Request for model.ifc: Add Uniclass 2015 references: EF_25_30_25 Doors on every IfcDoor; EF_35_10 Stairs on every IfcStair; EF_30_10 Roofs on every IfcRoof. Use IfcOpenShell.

First a look at what the model holds.

```python
import ifcopenshell

model = ifcopenshell.open("model.ifc")
print(model.schema)
print("classifications:", [c.Name for c in model.by_type("IfcClassification")])
for ifc_class in ("IfcDoor", "IfcRoof", "IfcStair", "IfcWall", "IfcWindow"):
    print(ifc_class, len(model.by_type(ifc_class)))
```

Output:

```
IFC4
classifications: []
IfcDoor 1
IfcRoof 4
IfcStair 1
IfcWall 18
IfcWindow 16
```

```python
import ifcopenshell
import ifcopenshell.api.classification

model = ifcopenshell.open("model.ifc")

system = ifcopenshell.api.classification.add_classification(model, classification="Uniclass 2015")

codes = {
    "IfcDoor": ("EF_25_30_25", "Doors"),
    "IfcStair": ("EF_35_10", "Stairs"),
    "IfcRoof": ("EF_30_10", "Roofs"),
}
for ifc_class, (code, name) in codes.items():
    products = model.by_type(ifc_class)
    ifcopenshell.api.classification.add_reference(
        model, products=products, classification=system, identification=code, name=name
    )
    print(code, len(products))

model.write("model_v2.ifc")
```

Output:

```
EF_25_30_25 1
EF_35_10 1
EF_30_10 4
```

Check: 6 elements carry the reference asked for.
